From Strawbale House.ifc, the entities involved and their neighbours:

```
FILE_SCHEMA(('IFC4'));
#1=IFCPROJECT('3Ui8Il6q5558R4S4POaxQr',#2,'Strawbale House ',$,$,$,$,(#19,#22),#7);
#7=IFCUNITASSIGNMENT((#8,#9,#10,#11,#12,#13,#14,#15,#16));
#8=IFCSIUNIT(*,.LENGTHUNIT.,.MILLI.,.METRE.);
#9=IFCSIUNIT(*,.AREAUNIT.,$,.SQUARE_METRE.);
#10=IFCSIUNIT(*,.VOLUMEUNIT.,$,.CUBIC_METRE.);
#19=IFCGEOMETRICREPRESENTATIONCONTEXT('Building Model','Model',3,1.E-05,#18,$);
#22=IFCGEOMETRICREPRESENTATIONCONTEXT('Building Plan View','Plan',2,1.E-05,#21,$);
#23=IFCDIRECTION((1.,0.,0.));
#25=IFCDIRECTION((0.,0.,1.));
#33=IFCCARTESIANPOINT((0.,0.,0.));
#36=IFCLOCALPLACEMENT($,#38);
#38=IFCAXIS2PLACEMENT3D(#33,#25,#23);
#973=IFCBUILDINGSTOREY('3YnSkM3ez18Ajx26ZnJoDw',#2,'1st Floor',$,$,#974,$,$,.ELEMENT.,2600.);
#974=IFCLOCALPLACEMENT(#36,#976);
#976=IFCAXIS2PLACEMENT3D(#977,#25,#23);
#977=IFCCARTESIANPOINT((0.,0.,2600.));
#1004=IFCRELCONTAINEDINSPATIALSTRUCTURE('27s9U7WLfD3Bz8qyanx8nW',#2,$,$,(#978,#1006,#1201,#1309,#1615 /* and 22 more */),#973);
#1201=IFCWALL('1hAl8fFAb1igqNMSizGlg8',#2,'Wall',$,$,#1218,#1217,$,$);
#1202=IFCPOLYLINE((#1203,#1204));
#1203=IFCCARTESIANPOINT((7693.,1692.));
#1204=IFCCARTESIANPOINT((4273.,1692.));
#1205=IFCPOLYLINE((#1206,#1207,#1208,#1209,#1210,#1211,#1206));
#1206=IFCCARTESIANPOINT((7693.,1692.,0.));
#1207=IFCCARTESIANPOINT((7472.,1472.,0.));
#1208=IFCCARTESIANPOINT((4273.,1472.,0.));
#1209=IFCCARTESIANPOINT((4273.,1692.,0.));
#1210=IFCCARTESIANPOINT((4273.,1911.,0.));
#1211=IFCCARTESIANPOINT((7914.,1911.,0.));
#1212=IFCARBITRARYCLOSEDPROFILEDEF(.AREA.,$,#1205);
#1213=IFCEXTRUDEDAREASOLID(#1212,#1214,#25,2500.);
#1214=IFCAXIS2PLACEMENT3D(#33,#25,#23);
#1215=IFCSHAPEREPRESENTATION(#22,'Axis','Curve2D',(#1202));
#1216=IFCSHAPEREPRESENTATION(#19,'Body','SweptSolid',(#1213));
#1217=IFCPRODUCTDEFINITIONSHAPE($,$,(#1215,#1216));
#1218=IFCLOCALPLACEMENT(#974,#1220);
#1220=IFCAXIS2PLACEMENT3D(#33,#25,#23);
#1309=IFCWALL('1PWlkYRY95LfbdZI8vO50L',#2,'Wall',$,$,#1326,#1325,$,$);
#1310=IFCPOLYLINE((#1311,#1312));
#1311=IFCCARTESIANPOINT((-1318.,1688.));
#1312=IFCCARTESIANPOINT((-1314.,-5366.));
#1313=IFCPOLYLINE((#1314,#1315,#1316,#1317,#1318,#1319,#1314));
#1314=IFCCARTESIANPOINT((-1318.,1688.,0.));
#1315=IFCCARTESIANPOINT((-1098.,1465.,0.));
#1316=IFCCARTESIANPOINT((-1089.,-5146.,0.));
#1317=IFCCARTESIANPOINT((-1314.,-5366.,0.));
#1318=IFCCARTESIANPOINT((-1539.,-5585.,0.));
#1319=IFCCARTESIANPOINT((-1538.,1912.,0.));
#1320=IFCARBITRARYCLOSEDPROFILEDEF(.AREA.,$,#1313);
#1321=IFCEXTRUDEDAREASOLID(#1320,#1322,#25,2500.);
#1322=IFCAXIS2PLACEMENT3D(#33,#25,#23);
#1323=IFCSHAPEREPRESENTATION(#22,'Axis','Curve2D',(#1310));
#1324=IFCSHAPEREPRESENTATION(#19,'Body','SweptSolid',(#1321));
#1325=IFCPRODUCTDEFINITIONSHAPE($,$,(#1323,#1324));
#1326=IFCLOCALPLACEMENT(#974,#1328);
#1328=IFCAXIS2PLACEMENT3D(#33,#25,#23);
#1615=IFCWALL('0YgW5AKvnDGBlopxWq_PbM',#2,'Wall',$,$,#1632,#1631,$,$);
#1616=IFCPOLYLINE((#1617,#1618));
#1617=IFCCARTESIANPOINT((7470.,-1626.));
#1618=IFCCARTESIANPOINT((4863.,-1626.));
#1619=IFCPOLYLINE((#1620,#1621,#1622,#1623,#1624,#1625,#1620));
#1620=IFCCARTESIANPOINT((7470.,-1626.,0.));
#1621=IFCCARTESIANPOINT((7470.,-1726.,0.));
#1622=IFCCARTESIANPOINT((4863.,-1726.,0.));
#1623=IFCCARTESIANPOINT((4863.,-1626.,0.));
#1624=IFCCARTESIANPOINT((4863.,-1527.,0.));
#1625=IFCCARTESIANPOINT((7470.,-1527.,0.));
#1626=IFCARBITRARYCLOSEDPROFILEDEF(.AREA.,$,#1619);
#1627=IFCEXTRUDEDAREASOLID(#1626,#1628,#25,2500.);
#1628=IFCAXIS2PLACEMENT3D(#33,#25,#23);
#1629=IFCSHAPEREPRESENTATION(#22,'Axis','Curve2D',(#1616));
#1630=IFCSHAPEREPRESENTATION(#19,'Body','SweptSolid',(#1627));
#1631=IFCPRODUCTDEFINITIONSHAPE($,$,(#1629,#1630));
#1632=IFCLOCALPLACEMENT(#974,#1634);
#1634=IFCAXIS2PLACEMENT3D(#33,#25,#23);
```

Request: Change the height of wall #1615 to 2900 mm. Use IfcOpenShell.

```python
import ifcopenshell
import ifcopenshell.geom
import ifcopenshell.util.shape
import ifcopenshell.util.unit

model = ifcopenshell.open("Strawbale House.ifc")
unit_scale = ifcopenshell.util.unit.calculate_unit_scale(model)
settings = ifcopenshell.geom.settings()


def volume(element):
    """Net volume in cubic metres, openings subtracted."""
    shape = ifcopenshell.geom.create_shape(settings, element)
    return ifcopenshell.util.shape.get_volume(shape.geometry)


wall = model.by_guid("0YgW5AKvnDGBlopxWq_PbM")
before = volume(wall)

body = next(r for r in wall.Representation.Representations if r.RepresentationIdentifier == "Body")
solid = body.Items[0]
old_height = solid.Depth
solid.Depth = 2.9 / unit_scale
after = volume(wall)

print(f"height {old_height:g} -> {solid.Depth:g}, volume {before:.3f} -> {after:.3f} m3")

model.write("Strawbale House_edited.ifc")
```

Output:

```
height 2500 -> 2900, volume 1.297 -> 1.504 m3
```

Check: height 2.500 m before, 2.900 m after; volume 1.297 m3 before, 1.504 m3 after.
